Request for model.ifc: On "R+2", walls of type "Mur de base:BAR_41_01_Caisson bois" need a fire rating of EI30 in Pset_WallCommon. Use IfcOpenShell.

First a look at what the model holds.

```python
import ifcopenshell
import ifcopenshell.util.element

model = ifcopenshell.open("model.ifc")
print(model.schema)
storey = next(s for s in model.by_type("IfcBuildingStorey") if s.Name == "R+2")
walls = [e for e in ifcopenshell.util.element.get_decomposition(storey) if e.is_a("IfcWall")]
seen = {}
for e in walls:
    element_type = ifcopenshell.util.element.get_type(e)
    key = (element_type.Name if element_type != e and element_type else None, ifcopenshell.util.element.get_pset(e, "Pset_WallCommon", "FireRating"))
    seen[key] = seen.get(key, 0) + 1
for (name, value), count in sorted(seen.items(), key=str):
    print(count, "x", name, "|", value)
```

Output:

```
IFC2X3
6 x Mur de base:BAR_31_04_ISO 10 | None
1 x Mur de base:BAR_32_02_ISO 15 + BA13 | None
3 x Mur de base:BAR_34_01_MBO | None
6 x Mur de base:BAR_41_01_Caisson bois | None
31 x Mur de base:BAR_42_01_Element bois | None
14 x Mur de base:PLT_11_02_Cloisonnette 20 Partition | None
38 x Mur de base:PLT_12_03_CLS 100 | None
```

```python
import ifcopenshell
import ifcopenshell.api.pset
import ifcopenshell.util.element

model = ifcopenshell.open("model.ifc")

storey = next(s for s in model.by_type("IfcBuildingStorey") if s.Name == "R+2")
walls = [e for e in ifcopenshell.util.element.get_decomposition(storey) if e.is_a("IfcWall")]

count = 0
for e in walls:
    element_type = ifcopenshell.util.element.get_type(e)
    if element_type in (None, e) or element_type.Name != "Mur de base:BAR_41_01_Caisson bois":
        continue
    # add_pset returns the element's existing set when there is one.
    pset = ifcopenshell.api.pset.add_pset(model, product=e, name="Pset_WallCommon")
    ifcopenshell.api.pset.edit_pset(model, pset=pset, properties={"FireRating": "EI30"})
    count += 1

print(count, "walls updated")

model.write("model_updated.ifc")
```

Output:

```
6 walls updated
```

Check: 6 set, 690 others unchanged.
